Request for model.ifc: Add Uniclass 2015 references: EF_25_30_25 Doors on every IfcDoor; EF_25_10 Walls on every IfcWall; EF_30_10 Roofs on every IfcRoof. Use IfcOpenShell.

First a look at what the model holds.

```python
import ifcopenshell

model = ifcopenshell.open("model.ifc")
print(model.schema)
print("classifications:", [c.Name for c in model.by_type("IfcClassification")])
for ifc_class in ("IfcDoor", "IfcRoof", "IfcStair", "IfcWall", "IfcWindow"):
    print(ifc_class, len(model.by_type(ifc_class)))
```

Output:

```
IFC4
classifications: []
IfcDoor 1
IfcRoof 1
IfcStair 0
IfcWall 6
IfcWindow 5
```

```python
import ifcopenshell
import ifcopenshell.api.classification

model = ifcopenshell.open("model.ifc")

system = ifcopenshell.api.classification.add_classification(model, classification="Uniclass 2015")

codes = {
    "IfcDoor": ("EF_25_30_25", "Doors"),
    "IfcWall": ("EF_25_10", "Walls"),
    "IfcRoof": ("EF_30_10", "Roofs"),
}
for ifc_class, (code, name) in codes.items():
    products = model.by_type(ifc_class)
    ifcopenshell.api.classification.add_reference(
        model, products=products, classification=system, identification=code, name=name
    )
    print(code, len(products))

model.write("model_updated.ifc")
```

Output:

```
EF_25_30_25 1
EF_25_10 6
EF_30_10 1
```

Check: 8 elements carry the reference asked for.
